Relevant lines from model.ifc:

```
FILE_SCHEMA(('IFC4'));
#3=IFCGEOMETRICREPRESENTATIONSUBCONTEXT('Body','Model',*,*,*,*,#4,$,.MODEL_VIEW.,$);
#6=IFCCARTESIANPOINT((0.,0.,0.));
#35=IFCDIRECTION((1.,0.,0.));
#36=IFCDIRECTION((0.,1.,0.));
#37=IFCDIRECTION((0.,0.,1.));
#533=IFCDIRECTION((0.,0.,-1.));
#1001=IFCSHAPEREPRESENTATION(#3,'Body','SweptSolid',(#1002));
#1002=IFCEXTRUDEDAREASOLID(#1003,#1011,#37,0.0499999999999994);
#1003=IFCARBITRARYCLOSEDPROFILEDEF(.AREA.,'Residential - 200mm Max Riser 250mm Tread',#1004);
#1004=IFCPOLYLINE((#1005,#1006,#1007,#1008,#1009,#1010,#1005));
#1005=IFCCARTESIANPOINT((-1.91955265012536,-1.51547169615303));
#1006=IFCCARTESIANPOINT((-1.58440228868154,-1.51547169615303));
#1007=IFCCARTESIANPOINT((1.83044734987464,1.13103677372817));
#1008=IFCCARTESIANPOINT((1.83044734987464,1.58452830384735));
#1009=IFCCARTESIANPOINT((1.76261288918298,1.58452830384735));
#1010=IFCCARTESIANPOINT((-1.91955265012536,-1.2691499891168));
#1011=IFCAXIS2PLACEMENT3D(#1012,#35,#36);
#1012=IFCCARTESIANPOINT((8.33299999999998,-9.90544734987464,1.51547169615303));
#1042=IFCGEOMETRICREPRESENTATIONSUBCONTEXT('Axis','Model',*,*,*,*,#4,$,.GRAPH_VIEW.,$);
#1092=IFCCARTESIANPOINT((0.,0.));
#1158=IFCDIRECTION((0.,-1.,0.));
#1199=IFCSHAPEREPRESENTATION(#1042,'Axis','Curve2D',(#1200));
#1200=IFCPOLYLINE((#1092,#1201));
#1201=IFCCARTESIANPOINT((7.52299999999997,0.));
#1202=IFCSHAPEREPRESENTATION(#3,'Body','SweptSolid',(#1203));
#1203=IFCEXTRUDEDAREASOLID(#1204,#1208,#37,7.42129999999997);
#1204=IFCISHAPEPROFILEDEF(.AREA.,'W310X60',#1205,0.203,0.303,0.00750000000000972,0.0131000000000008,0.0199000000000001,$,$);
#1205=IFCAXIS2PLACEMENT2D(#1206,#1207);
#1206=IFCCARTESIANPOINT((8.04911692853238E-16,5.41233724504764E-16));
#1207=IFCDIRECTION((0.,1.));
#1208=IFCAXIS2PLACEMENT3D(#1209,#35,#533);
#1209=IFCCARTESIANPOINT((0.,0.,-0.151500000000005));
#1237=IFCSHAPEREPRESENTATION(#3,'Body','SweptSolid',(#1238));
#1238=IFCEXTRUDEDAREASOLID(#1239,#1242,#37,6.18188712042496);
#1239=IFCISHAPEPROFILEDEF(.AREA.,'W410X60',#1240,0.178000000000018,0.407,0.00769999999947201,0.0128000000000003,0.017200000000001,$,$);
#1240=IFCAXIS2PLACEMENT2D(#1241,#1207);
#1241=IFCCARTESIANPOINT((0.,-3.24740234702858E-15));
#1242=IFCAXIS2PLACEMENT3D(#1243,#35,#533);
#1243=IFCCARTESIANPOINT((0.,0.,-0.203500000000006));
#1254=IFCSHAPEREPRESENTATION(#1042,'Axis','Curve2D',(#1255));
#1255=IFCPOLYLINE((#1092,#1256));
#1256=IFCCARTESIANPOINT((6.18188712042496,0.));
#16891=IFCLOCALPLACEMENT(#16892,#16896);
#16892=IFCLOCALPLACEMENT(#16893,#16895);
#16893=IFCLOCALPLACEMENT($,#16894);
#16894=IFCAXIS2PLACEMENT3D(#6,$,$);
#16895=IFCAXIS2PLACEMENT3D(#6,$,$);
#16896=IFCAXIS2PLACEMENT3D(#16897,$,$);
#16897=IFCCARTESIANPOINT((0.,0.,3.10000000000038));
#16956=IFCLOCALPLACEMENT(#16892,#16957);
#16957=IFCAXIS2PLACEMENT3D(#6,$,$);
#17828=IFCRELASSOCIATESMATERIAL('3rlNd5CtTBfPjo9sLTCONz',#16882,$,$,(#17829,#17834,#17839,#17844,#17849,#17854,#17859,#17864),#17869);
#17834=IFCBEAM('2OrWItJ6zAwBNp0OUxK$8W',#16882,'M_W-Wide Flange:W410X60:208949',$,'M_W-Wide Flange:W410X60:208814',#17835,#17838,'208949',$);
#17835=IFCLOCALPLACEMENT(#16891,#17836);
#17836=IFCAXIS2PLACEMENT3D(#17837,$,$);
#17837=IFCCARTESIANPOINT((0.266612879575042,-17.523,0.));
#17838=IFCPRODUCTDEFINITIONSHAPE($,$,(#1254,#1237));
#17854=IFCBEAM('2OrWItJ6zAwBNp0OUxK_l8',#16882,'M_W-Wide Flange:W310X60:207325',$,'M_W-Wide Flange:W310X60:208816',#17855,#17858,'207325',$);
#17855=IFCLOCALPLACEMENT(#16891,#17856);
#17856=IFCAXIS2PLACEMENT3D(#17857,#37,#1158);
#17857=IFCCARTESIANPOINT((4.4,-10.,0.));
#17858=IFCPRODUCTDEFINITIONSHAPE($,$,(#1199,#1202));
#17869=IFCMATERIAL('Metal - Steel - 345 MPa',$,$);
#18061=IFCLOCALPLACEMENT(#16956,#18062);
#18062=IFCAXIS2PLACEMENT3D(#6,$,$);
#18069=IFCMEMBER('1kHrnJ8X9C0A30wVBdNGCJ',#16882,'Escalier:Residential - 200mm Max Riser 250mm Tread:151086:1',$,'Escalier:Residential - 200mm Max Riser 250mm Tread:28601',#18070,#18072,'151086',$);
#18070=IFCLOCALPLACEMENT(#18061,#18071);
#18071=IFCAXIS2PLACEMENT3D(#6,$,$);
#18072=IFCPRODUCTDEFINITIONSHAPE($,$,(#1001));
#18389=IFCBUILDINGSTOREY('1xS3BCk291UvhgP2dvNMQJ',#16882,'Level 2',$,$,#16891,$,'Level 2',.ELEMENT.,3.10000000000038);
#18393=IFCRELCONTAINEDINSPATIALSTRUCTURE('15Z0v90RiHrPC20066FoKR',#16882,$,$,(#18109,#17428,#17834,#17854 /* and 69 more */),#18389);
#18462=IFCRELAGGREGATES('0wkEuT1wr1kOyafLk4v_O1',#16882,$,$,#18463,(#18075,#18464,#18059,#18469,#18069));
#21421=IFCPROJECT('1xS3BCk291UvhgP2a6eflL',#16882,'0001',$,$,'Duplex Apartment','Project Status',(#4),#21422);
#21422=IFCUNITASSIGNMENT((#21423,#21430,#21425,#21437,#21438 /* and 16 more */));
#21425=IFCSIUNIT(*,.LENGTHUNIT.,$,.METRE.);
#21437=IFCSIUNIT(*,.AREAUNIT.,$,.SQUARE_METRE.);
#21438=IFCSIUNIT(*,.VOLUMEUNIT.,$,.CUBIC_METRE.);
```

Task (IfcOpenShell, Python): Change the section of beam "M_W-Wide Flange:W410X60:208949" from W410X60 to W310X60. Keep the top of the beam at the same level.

```python
import ifcopenshell
import ifcopenshell.util.element
import ifcopenshell.util.representation

model = ifcopenshell.open("model.ifc")

member = model.by_guid("2OrWItJ6zAwBNp0OUxK$8W")
source = next(p for p in model.by_type("IfcIShapeProfileDef") if p.ProfileName == "W310X60")

body = ifcopenshell.util.representation.get_representation(member, "Model", "Body")
solid = body.Items[0]
old_profile = solid.SweptArea

# Copy the section's sizes but keep this member's own profile position.
profile = ifcopenshell.util.element.copy(model, source)
# Profiles are centred, so shift by half the change in depth to hold the top.
shift = (old_profile.OverallDepth - profile.OverallDepth) / 2
x, y = old_profile.Position.Location.Coordinates
up = (-1.0, 0.0)  # upwards, in the solid's own plane
location = model.createIfcCartesianPoint((x + up[0] * shift, y + up[1] * shift))
profile.Position = model.createIfcAxis2Placement2D(location, old_profile.Position.RefDirection)
solid.SweptArea = profile
if not model.get_total_inverses(old_profile):
    ifcopenshell.util.element.remove_deep2(model, old_profile)
member.Name = member.Name.replace("W410X60", "W310X60")
member.ObjectType = member.ObjectType.replace("W410X60", "W310X60")

print(solid.SweptArea)

model.write("model_rev.ifc")
```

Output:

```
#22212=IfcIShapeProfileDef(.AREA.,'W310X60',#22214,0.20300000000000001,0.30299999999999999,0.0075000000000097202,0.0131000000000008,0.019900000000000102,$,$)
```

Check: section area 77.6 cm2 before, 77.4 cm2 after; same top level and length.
